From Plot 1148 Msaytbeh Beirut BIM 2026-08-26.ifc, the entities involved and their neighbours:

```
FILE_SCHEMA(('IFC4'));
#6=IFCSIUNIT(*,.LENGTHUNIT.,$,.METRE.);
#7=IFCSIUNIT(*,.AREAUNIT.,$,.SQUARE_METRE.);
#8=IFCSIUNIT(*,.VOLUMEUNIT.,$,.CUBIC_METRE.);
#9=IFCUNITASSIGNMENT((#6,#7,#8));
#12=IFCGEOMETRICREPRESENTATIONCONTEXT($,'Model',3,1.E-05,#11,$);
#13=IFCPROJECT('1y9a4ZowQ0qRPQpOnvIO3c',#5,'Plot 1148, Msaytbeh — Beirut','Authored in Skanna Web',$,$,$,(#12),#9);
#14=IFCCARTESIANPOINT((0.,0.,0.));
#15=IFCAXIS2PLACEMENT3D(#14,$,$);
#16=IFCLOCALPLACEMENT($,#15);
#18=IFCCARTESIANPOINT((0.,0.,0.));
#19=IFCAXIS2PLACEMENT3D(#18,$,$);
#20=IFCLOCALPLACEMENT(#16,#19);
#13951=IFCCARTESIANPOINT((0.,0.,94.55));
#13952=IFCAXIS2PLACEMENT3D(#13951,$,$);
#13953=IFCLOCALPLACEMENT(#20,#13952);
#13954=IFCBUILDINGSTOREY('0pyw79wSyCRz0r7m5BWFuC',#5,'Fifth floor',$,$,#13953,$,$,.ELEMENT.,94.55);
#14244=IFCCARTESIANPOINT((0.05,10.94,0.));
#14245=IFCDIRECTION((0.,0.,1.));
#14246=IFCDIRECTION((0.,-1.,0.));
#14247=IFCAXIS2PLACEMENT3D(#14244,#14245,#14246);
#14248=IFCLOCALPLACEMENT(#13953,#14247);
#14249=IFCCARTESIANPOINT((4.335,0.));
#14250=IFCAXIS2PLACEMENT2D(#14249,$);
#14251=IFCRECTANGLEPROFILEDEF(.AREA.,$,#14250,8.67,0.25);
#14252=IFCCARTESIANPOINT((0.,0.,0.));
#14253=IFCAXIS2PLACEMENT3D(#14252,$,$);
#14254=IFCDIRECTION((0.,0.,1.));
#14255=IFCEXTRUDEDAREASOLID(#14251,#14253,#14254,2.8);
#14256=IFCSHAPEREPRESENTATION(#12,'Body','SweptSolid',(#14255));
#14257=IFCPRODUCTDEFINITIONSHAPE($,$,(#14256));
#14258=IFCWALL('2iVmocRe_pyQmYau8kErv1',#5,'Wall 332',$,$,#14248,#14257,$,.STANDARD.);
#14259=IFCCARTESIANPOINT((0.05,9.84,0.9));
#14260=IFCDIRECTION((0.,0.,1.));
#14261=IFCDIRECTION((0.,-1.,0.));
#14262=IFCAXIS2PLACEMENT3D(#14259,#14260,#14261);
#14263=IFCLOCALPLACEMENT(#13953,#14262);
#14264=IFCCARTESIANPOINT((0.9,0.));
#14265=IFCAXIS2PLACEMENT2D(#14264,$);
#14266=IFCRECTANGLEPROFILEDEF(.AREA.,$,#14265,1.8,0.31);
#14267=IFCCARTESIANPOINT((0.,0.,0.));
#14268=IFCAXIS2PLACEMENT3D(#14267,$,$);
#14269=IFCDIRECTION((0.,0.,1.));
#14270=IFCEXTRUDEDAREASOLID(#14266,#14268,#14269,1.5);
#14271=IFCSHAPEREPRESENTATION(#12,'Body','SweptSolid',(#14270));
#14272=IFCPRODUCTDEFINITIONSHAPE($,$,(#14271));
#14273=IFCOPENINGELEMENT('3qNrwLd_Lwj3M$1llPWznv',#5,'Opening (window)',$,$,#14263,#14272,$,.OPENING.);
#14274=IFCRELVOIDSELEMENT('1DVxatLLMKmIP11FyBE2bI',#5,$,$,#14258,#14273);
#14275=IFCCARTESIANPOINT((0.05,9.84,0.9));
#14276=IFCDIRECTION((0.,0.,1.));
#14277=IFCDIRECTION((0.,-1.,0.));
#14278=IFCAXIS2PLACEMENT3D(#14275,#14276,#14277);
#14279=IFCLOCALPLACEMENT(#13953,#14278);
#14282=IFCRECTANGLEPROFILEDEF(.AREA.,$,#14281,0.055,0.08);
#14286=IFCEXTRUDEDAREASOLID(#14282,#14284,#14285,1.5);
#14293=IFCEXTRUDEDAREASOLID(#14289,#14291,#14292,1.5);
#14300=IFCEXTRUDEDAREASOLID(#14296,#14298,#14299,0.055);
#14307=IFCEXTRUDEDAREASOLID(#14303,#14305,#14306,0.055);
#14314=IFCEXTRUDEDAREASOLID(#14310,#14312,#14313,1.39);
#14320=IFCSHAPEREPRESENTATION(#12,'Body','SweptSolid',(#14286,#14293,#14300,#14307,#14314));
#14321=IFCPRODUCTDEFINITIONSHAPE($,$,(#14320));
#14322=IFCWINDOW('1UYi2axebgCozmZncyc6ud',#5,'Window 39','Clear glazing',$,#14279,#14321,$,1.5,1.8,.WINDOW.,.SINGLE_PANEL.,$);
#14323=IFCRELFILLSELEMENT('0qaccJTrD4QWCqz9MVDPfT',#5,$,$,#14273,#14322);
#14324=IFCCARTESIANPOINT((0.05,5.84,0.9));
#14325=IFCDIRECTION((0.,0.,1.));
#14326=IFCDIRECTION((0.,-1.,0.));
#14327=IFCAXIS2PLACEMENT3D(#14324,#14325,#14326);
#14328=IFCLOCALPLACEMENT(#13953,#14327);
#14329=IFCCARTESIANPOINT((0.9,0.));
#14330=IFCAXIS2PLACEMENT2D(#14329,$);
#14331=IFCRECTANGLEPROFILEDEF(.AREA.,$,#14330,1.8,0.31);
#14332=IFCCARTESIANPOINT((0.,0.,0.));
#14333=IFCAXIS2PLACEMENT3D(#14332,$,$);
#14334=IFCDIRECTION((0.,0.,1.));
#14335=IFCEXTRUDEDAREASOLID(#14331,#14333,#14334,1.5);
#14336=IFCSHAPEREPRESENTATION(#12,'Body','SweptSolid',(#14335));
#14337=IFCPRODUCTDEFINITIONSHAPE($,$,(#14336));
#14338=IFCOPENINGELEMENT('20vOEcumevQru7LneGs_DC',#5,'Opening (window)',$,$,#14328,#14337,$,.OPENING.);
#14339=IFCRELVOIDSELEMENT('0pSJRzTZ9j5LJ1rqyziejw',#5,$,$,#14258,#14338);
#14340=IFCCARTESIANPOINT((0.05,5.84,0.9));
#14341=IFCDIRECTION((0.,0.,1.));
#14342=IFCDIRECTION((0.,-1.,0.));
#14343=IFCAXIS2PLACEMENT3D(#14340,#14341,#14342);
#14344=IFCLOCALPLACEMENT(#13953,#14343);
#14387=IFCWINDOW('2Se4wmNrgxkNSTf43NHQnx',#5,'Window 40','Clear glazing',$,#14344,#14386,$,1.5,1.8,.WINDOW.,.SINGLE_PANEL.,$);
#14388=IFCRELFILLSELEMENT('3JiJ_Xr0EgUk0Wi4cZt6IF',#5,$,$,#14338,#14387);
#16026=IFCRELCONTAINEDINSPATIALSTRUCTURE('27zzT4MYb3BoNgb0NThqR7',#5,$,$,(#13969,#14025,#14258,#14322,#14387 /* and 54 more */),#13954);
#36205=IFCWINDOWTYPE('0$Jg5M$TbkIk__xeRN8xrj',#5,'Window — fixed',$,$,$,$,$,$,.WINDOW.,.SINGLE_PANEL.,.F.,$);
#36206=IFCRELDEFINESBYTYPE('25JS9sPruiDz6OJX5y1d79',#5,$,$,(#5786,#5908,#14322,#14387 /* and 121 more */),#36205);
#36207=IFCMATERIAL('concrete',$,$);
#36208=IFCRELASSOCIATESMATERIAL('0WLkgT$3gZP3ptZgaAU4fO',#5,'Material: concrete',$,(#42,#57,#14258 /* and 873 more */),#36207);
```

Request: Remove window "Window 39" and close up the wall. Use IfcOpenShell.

```python
import ifcopenshell
import ifcopenshell.api.feature
import ifcopenshell.api.root
import ifcopenshell.geom
import ifcopenshell.util.shape

model = ifcopenshell.open("Plot 1148 Msaytbeh Beirut BIM 2026-08-26.ifc")
settings = ifcopenshell.geom.settings()


def volume(element):
    """Net volume in cubic metres, openings subtracted."""
    shape = ifcopenshell.geom.create_shape(settings, element)
    return ifcopenshell.util.shape.get_volume(shape.geometry)


window = model.by_guid("1UYi2axebgCozmZncyc6ud")
opening = window.FillsVoids[0].RelatingOpeningElement
wall = opening.VoidsElements[0].RelatingBuildingElement
before = volume(wall)

ifcopenshell.api.root.remove_product(model, product=window)
ifcopenshell.api.feature.remove_feature(model, feature=opening)

after = volume(wall)

print(f"wall volume {before:.3f} -> {after:.3f} m3")

model.write("Plot 1148 Msaytbeh Beirut BIM 2026-08-26-out.ifc")
```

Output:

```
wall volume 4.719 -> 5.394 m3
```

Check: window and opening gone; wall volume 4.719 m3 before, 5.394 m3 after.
